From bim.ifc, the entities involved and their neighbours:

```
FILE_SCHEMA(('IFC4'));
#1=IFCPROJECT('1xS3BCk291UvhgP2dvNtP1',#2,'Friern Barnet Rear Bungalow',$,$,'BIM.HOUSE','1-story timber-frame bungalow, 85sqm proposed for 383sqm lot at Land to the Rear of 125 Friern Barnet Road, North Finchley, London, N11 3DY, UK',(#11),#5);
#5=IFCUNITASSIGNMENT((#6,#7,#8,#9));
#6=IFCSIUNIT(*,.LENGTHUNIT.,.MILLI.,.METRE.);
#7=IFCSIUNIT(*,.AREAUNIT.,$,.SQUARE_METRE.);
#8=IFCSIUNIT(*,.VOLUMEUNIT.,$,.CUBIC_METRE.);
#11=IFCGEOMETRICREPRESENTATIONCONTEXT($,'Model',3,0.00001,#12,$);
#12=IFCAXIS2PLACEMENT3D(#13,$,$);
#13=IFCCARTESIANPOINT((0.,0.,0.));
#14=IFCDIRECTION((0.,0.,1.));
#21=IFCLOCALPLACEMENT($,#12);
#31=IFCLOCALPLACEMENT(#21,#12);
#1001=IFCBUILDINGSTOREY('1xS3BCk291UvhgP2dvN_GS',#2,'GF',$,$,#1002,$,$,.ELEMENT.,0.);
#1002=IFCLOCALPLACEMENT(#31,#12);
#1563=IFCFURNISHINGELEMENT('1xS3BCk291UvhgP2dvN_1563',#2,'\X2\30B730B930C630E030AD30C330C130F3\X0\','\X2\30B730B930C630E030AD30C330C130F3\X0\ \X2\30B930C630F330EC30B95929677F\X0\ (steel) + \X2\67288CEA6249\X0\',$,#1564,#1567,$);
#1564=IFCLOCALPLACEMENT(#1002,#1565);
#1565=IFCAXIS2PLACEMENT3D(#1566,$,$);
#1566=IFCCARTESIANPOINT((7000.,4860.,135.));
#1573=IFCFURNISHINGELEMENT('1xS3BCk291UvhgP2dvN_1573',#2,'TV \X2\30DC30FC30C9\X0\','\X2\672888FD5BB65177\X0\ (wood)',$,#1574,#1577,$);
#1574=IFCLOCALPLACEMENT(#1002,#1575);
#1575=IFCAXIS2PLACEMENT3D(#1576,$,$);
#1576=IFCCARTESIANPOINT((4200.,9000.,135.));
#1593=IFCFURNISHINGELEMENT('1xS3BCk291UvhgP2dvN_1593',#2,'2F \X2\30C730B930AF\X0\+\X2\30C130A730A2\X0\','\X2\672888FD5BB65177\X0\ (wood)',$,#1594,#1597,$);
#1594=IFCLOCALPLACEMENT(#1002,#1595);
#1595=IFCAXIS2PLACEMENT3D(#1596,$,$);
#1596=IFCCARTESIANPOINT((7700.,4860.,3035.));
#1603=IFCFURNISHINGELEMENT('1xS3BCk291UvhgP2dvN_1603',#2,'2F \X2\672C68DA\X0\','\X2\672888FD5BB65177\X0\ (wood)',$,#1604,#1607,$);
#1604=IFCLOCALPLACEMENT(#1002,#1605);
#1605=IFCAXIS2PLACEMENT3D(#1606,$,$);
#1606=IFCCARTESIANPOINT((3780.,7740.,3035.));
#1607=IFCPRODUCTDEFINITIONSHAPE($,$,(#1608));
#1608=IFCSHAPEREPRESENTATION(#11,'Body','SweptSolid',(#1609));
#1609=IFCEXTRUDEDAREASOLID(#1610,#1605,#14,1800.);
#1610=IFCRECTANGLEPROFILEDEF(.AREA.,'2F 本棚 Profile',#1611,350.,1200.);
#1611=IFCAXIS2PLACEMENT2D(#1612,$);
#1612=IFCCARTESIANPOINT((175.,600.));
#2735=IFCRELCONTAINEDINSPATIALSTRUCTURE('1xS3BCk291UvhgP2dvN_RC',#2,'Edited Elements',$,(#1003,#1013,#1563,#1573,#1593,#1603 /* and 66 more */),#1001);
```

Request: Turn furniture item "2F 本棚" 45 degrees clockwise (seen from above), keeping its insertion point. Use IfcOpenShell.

```python
import ifcopenshell
import ifcopenshell.api.geometry
import ifcopenshell.util.placement

model = ifcopenshell.open("bim.ifc")

item = model.by_id(1603)
matrix = ifcopenshell.util.placement.get_local_placement(item.ObjectPlacement)
matrix = matrix @ ifcopenshell.util.placement.rotation(-45, "Z")
ifcopenshell.api.geometry.edit_object_placement(model, product=item, matrix=matrix, is_si=False)

print(ifcopenshell.util.placement.get_local_placement(item.ObjectPlacement).round(3) + 0.0)

model.write("bim_v2.ifc")
```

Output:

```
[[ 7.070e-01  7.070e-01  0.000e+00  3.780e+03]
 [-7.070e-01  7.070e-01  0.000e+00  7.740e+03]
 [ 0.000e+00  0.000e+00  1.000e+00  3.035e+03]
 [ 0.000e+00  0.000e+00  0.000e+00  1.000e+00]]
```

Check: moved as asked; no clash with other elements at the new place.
